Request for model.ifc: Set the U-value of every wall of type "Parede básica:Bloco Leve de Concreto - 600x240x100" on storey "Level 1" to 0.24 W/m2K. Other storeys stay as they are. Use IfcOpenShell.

First a look at what the model holds.

```python
import ifcopenshell
import ifcopenshell.util.element

model = ifcopenshell.open("model.ifc")
print(model.schema)
storey = next(s for s in model.by_type("IfcBuildingStorey") if s.Name == "Level 1")
walls = [e for e in ifcopenshell.util.element.get_decomposition(storey) if e.is_a("IfcWall")]
seen = {}
for e in walls:
    element_type = ifcopenshell.util.element.get_type(e)
    key = (element_type.Name if element_type != e and element_type else None, ifcopenshell.util.element.get_pset(e, "Pset_WallCommon", "ThermalTransmittance"))
    seen[key] = seen.get(key, 0) + 1
for (name, value), count in sorted(seen.items(), key=str):
    print(count, "x", name, "|", value)
```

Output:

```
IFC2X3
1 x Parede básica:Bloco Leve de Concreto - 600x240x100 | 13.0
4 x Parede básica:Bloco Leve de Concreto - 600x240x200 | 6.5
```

```python
import ifcopenshell
import ifcopenshell.api.pset
import ifcopenshell.util.element

model = ifcopenshell.open("model.ifc")

storey = next(s for s in model.by_type("IfcBuildingStorey") if s.Name == "Level 1")
walls = [e for e in ifcopenshell.util.element.get_decomposition(storey) if e.is_a("IfcWall")]

count = 0
for e in walls:
    element_type = ifcopenshell.util.element.get_type(e)
    if element_type in (None, e) or element_type.Name != "Parede básica:Bloco Leve de Concreto - 600x240x100":
        continue
    # add_pset returns the element's existing set when there is one.
    pset = ifcopenshell.api.pset.add_pset(model, product=e, name="Pset_WallCommon")
    ifcopenshell.api.pset.edit_pset(model, pset=pset, properties={"ThermalTransmittance": 0.24})
    count += 1

print(count, "walls updated")

model.write("model_v2.ifc")
```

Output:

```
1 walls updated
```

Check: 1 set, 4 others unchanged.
